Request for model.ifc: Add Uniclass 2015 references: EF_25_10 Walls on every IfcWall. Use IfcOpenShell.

First a look at what the model holds.

```python
import ifcopenshell

model = ifcopenshell.open("model.ifc")
print(model.schema)
print("classifications:", [c.Name for c in model.by_type("IfcClassification")])
for ifc_class in ("IfcDoor", "IfcRoof", "IfcStair", "IfcWall", "IfcWindow"):
    print(ifc_class, len(model.by_type(ifc_class)))
```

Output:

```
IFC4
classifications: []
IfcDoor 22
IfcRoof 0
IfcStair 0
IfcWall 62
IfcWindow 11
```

```python
import ifcopenshell
import ifcopenshell.api.classification

model = ifcopenshell.open("model.ifc")

system = ifcopenshell.api.classification.add_classification(model, classification="Uniclass 2015")

codes = {
    "IfcWall": ("EF_25_10", "Walls"),
}
for ifc_class, (code, name) in codes.items():
    products = model.by_type(ifc_class)
    ifcopenshell.api.classification.add_reference(
        model, products=products, classification=system, identification=code, name=name
    )
    print(code, len(products))

model.write("model_v2.ifc")
```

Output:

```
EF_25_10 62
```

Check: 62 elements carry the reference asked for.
